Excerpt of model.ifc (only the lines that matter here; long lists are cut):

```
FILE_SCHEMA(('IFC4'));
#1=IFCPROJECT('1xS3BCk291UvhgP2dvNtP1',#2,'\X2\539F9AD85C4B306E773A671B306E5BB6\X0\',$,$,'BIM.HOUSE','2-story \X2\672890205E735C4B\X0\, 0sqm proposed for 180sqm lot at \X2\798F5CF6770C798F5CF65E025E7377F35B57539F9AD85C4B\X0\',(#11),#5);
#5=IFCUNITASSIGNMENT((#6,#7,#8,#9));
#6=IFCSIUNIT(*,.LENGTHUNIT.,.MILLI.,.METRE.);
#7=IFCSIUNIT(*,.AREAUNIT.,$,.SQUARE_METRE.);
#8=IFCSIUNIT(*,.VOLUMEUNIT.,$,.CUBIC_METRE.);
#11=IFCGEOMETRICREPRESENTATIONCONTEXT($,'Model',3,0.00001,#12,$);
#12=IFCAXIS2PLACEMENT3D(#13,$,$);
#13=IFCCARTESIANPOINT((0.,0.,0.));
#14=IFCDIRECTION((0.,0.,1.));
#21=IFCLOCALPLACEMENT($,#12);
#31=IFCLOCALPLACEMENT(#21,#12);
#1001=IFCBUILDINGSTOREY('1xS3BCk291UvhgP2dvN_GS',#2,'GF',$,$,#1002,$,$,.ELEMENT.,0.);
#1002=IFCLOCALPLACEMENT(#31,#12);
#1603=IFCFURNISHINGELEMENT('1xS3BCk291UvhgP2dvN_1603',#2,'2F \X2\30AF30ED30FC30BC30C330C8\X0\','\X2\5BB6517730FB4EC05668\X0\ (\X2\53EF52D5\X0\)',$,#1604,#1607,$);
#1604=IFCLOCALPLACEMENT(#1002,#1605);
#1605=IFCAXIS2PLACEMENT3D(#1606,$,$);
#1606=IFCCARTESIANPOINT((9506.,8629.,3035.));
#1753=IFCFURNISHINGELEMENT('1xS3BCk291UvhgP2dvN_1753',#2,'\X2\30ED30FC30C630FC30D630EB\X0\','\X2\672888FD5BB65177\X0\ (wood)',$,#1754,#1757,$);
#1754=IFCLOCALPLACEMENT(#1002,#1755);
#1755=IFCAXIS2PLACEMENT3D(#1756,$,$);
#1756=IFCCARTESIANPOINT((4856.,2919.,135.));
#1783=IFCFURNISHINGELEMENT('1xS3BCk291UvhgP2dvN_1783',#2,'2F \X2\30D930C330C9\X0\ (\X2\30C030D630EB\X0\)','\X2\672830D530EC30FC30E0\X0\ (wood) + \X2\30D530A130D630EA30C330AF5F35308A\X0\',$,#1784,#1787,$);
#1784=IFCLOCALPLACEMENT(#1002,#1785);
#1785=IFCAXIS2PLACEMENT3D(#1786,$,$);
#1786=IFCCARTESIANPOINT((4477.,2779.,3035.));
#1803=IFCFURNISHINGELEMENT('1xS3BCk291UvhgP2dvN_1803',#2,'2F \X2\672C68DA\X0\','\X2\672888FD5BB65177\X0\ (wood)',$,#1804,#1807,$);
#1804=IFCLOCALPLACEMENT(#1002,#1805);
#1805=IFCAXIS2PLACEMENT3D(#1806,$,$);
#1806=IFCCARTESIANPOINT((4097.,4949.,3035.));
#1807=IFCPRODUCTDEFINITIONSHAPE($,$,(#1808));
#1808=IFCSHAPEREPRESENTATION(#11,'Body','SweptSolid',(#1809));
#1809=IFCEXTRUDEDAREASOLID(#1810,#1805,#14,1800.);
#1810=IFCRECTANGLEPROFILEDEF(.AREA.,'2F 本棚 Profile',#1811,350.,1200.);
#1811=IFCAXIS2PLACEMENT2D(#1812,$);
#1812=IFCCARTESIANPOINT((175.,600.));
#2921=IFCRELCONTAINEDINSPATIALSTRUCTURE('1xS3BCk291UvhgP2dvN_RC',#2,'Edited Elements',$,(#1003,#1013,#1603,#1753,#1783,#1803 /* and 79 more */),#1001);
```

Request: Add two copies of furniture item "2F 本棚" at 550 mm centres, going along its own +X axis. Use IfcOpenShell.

```python
import ifcopenshell
import ifcopenshell.api.geometry
import ifcopenshell.api.root
import ifcopenshell.util.element
import ifcopenshell.util.placement
import ifcopenshell.util.unit

model = ifcopenshell.open("model.ifc")
unit_scale = ifcopenshell.util.unit.calculate_unit_scale(model)


def reuse_history(source, copy):
    """copy_class also copies each property set's owner history, people and application; keep the originals."""
    for rel in copy.IsDefinedBy:
        if rel.is_a("IfcRelDefinesByProperties") and (history := rel.RelatingPropertyDefinition.OwnerHistory):
            rel.RelatingPropertyDefinition.OwnerHistory = source.OwnerHistory
            ifcopenshell.util.element.remove_deep2(model, history)


source = model.by_guid("1xS3BCk291UvhgP2dvN_1803")
base = ifcopenshell.util.placement.get_local_placement(source.ObjectPlacement)
step = base[:3, 0] * 0.55 / unit_scale

for i in range(1, 3):
    copy = ifcopenshell.api.root.copy_class(model, product=source)
    copy.Representation = ifcopenshell.util.element.copy_deep(
        model, source.Representation, exclude=["IfcGeometricRepresentationContext", "IfcRepresentationMap"]
    )
    reuse_history(source, copy)
    matrix = base.copy()
    matrix[:3, 3] += i * step
    print("added at", matrix[:3, 3].round(3) + 0.0)
    ifcopenshell.api.geometry.edit_object_placement(model, product=copy, matrix=matrix, is_si=False)

model.write("model_updated.ifc")
```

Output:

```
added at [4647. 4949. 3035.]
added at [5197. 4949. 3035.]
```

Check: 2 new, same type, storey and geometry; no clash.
